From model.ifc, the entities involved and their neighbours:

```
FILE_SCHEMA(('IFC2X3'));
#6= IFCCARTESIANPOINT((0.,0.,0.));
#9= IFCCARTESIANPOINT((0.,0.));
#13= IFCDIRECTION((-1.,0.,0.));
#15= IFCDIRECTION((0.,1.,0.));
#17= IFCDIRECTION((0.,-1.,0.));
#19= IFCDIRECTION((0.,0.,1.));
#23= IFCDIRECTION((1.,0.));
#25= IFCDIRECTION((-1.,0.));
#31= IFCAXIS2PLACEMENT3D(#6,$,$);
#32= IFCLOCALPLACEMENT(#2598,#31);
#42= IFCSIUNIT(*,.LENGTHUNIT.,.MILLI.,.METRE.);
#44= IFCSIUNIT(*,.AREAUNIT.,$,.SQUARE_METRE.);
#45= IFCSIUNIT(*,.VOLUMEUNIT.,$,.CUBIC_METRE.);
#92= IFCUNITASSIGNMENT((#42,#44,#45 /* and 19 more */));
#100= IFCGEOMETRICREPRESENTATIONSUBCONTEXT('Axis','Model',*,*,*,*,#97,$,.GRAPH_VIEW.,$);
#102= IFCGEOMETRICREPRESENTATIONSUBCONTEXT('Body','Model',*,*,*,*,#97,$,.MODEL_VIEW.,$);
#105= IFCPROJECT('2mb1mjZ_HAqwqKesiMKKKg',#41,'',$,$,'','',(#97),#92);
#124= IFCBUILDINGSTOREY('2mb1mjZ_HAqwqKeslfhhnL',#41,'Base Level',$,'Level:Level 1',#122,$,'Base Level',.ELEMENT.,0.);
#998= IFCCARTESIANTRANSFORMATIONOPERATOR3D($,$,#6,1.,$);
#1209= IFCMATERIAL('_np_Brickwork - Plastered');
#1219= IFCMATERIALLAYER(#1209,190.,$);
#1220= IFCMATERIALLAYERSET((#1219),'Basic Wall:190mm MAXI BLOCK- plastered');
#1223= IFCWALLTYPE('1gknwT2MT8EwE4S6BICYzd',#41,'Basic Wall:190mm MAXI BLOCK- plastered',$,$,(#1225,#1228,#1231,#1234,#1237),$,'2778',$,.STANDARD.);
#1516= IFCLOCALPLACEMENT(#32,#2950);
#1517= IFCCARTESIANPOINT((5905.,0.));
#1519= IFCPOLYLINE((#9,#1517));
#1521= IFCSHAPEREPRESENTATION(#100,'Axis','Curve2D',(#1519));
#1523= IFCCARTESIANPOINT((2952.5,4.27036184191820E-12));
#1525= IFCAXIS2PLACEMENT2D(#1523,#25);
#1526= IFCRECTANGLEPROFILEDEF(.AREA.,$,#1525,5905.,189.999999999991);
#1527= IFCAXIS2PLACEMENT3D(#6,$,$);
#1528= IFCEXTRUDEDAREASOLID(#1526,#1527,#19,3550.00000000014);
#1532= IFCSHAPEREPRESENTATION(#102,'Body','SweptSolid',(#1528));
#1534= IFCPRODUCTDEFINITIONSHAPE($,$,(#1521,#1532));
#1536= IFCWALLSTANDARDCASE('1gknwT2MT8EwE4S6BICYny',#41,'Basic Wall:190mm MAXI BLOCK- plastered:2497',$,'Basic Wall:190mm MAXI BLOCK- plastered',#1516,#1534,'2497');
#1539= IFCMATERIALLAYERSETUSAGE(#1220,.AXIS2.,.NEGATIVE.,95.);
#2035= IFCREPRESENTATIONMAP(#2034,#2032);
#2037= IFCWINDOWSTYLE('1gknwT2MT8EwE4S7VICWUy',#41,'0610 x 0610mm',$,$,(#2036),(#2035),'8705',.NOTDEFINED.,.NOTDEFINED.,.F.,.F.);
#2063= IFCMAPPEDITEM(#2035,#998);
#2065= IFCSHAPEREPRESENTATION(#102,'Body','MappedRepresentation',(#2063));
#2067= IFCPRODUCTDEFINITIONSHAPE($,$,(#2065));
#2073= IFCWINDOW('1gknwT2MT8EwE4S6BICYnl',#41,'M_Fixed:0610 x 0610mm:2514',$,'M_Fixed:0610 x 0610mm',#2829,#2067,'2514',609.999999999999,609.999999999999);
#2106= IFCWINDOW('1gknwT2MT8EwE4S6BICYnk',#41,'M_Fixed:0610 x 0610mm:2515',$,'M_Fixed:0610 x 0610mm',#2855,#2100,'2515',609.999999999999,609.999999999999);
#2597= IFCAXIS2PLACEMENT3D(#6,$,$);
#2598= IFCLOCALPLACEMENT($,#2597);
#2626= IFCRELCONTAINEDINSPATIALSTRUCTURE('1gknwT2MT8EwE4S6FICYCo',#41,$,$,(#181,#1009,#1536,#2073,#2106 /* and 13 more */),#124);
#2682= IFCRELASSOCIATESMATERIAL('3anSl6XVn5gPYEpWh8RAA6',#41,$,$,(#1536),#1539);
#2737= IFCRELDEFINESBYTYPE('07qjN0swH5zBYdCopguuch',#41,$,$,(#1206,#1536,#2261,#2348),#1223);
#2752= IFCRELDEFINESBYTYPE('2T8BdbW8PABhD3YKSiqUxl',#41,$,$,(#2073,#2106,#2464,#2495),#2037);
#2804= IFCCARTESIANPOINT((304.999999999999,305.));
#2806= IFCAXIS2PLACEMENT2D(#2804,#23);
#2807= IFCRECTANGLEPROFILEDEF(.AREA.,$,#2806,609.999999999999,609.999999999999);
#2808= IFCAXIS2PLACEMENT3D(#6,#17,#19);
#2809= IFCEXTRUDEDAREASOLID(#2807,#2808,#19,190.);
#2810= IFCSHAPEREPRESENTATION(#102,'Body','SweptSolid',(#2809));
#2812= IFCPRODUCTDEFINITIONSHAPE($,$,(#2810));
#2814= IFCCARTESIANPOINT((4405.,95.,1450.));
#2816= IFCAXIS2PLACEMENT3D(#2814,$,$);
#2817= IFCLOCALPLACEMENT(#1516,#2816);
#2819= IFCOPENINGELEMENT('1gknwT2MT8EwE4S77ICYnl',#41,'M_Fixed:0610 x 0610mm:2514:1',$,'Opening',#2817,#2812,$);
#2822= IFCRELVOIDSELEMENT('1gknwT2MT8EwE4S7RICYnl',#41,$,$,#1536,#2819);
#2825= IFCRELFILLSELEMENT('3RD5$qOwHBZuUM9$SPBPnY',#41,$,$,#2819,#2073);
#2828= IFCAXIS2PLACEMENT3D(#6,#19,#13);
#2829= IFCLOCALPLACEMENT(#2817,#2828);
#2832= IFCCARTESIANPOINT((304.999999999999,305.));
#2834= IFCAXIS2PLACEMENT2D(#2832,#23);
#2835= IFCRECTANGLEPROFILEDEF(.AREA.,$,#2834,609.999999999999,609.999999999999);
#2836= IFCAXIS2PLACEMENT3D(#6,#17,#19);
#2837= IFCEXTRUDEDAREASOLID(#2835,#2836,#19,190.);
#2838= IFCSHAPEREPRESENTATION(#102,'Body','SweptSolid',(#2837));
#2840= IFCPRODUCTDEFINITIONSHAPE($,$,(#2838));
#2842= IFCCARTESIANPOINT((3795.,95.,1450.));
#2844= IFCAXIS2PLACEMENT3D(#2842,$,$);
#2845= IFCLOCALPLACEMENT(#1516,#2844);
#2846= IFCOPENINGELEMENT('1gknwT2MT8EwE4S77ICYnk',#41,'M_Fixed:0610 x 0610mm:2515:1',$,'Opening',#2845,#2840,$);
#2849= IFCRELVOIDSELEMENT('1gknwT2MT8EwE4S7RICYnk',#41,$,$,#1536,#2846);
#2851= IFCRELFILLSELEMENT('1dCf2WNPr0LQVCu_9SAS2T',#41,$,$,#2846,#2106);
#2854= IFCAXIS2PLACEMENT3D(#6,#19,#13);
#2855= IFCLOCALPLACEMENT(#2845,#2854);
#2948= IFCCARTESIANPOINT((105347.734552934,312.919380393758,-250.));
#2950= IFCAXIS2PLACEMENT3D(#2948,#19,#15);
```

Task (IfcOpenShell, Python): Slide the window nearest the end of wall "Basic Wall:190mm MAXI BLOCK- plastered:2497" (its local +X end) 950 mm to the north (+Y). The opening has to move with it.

```python
import ifcopenshell
import ifcopenshell.api.geometry
import ifcopenshell.util.placement
import ifcopenshell.util.unit

model = ifcopenshell.open("model.ifc")
unit_scale = ifcopenshell.util.unit.calculate_unit_scale(model)

window = model.by_guid("1gknwT2MT8EwE4S6BICYnl")
opening = window.FillsVoids[0].RelatingOpeningElement
wall = opening.VoidsElements[0].RelatingBuildingElement

wall_matrix = ifcopenshell.util.placement.get_local_placement(wall.ObjectPlacement)
shift = wall_matrix[:3, 0] * 0.95 / unit_scale
before = ifcopenshell.util.placement.get_local_placement(window.ObjectPlacement)[:3, 3].copy()

# The window is placed relative to its opening, so it follows when the opening moves.
matrix = ifcopenshell.util.placement.get_local_placement(opening.ObjectPlacement)
matrix[:3, 3] += shift
ifcopenshell.api.geometry.edit_object_placement(
    model, product=opening, matrix=matrix, is_si=False, should_transform_children=True
)

after = ifcopenshell.util.placement.get_local_placement(window.ObjectPlacement)[:3, 3]
print("window moved by", (after - before).round(3) + 0.0)

model.write("model_updated.ifc")
```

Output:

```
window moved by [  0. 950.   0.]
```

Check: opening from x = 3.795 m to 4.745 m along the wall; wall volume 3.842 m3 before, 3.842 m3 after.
